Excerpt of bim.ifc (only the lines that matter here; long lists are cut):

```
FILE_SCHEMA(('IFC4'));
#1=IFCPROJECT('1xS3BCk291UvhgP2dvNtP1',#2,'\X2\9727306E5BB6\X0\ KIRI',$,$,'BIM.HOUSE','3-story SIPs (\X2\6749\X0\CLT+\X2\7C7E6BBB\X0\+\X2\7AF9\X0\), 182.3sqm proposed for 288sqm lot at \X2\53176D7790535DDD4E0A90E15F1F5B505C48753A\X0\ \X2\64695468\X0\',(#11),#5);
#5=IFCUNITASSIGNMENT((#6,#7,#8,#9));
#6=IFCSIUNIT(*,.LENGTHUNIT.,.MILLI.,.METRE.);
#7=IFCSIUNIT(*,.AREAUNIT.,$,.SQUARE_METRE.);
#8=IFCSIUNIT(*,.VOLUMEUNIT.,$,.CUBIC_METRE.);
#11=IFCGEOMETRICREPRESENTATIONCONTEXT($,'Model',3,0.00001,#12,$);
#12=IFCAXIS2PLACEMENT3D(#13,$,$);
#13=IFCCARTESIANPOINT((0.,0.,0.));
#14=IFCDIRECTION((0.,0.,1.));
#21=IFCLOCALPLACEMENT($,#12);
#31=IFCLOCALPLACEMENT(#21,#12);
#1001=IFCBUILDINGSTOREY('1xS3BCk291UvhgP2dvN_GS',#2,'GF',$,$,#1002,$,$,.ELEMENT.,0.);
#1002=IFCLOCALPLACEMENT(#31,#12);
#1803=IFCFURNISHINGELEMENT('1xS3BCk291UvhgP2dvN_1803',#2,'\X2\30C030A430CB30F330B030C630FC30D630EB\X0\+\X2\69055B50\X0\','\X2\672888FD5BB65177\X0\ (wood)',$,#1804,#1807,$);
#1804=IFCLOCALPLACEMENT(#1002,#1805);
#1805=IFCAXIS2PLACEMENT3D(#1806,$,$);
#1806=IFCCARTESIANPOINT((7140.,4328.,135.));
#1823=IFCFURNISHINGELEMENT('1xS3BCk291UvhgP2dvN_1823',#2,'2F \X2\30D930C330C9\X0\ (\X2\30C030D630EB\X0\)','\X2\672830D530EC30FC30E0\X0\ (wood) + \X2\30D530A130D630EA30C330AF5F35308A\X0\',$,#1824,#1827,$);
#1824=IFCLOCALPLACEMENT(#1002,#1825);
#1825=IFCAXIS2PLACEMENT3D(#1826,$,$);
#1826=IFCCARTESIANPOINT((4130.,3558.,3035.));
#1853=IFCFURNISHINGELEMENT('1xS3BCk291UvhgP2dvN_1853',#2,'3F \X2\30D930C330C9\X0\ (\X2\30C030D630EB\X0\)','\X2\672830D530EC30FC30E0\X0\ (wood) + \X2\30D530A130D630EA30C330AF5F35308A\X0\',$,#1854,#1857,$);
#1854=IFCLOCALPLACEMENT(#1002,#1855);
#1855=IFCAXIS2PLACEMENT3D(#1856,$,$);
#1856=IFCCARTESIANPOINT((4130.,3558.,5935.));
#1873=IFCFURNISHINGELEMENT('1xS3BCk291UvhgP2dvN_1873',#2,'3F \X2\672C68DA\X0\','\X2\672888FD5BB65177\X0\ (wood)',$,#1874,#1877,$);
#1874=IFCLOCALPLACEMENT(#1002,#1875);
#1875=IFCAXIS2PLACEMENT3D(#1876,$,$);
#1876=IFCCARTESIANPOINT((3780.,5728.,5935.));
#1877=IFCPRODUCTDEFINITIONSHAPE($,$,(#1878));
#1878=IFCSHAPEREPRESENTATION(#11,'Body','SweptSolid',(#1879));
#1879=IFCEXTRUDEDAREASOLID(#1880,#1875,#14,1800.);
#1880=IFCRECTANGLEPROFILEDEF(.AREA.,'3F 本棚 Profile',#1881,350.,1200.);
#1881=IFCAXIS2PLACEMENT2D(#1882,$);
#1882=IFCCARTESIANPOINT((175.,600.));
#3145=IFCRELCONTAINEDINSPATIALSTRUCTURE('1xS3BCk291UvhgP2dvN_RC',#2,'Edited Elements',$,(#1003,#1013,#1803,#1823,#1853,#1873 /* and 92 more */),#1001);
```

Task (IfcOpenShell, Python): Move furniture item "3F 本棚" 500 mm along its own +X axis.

```python
import ifcopenshell
import ifcopenshell.api.geometry
import ifcopenshell.util.placement
import ifcopenshell.util.unit

model = ifcopenshell.open("bim.ifc")
unit_scale = ifcopenshell.util.unit.calculate_unit_scale(model)

item = model.by_id(1873)
matrix = ifcopenshell.util.placement.get_local_placement(item.ObjectPlacement)
matrix[:3, 3] += matrix[:3, 0] * 0.5 / unit_scale
ifcopenshell.api.geometry.edit_object_placement(model, product=item, matrix=matrix, is_si=False)

print(ifcopenshell.util.placement.get_local_placement(item.ObjectPlacement).round(3) + 0.0)

model.write("bim-out.ifc")
```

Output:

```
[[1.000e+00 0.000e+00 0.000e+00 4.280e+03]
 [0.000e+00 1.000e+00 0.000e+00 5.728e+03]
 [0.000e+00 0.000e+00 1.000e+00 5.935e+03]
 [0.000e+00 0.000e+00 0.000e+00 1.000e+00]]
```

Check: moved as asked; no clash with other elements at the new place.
